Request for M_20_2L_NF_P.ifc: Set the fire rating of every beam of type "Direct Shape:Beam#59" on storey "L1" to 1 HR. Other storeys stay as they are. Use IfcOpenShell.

First a look at what the model holds.

```python
import ifcopenshell
import ifcopenshell.util.element

model = ifcopenshell.open("M_20_2L_NF_P.ifc")
print(model.schema)
storey = next(s for s in model.by_type("IfcBuildingStorey") if s.Name == "L1")
beams = [e for e in ifcopenshell.util.element.get_decomposition(storey) if e.is_a("IfcBeam")]
seen = {}
for e in beams:
    element_type = ifcopenshell.util.element.get_type(e)
    key = (element_type.Name if element_type != e and element_type else None, ifcopenshell.util.element.get_pset(e, "Pset_BeamCommon", "FireRating"))
    seen[key] = seen.get(key, 0) + 1
for (name, value), count in sorted(seen.items(), key=str):
    print(count, "x", name, "|", value)
```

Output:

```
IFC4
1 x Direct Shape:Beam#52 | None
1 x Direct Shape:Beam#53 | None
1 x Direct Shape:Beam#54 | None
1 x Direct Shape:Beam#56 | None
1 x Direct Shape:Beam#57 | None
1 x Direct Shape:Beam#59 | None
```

```python
import ifcopenshell
import ifcopenshell.api.pset
import ifcopenshell.util.element

model = ifcopenshell.open("M_20_2L_NF_P.ifc")

storey = next(s for s in model.by_type("IfcBuildingStorey") if s.Name == "L1")
beams = [e for e in ifcopenshell.util.element.get_decomposition(storey) if e.is_a("IfcBeam")]

count = 0
for e in beams:
    element_type = ifcopenshell.util.element.get_type(e)
    if element_type in (None, e) or element_type.Name != "Direct Shape:Beam#59":
        continue
    # add_pset returns the element's existing set when there is one.
    pset = ifcopenshell.api.pset.add_pset(model, product=e, name="Pset_BeamCommon")
    ifcopenshell.api.pset.edit_pset(model, pset=pset, properties={"FireRating": "1 HR"})
    count += 1

print(count, "beams updated")

model.write("M_20_2L_NF_P_rev.ifc")
```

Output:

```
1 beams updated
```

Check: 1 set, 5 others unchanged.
